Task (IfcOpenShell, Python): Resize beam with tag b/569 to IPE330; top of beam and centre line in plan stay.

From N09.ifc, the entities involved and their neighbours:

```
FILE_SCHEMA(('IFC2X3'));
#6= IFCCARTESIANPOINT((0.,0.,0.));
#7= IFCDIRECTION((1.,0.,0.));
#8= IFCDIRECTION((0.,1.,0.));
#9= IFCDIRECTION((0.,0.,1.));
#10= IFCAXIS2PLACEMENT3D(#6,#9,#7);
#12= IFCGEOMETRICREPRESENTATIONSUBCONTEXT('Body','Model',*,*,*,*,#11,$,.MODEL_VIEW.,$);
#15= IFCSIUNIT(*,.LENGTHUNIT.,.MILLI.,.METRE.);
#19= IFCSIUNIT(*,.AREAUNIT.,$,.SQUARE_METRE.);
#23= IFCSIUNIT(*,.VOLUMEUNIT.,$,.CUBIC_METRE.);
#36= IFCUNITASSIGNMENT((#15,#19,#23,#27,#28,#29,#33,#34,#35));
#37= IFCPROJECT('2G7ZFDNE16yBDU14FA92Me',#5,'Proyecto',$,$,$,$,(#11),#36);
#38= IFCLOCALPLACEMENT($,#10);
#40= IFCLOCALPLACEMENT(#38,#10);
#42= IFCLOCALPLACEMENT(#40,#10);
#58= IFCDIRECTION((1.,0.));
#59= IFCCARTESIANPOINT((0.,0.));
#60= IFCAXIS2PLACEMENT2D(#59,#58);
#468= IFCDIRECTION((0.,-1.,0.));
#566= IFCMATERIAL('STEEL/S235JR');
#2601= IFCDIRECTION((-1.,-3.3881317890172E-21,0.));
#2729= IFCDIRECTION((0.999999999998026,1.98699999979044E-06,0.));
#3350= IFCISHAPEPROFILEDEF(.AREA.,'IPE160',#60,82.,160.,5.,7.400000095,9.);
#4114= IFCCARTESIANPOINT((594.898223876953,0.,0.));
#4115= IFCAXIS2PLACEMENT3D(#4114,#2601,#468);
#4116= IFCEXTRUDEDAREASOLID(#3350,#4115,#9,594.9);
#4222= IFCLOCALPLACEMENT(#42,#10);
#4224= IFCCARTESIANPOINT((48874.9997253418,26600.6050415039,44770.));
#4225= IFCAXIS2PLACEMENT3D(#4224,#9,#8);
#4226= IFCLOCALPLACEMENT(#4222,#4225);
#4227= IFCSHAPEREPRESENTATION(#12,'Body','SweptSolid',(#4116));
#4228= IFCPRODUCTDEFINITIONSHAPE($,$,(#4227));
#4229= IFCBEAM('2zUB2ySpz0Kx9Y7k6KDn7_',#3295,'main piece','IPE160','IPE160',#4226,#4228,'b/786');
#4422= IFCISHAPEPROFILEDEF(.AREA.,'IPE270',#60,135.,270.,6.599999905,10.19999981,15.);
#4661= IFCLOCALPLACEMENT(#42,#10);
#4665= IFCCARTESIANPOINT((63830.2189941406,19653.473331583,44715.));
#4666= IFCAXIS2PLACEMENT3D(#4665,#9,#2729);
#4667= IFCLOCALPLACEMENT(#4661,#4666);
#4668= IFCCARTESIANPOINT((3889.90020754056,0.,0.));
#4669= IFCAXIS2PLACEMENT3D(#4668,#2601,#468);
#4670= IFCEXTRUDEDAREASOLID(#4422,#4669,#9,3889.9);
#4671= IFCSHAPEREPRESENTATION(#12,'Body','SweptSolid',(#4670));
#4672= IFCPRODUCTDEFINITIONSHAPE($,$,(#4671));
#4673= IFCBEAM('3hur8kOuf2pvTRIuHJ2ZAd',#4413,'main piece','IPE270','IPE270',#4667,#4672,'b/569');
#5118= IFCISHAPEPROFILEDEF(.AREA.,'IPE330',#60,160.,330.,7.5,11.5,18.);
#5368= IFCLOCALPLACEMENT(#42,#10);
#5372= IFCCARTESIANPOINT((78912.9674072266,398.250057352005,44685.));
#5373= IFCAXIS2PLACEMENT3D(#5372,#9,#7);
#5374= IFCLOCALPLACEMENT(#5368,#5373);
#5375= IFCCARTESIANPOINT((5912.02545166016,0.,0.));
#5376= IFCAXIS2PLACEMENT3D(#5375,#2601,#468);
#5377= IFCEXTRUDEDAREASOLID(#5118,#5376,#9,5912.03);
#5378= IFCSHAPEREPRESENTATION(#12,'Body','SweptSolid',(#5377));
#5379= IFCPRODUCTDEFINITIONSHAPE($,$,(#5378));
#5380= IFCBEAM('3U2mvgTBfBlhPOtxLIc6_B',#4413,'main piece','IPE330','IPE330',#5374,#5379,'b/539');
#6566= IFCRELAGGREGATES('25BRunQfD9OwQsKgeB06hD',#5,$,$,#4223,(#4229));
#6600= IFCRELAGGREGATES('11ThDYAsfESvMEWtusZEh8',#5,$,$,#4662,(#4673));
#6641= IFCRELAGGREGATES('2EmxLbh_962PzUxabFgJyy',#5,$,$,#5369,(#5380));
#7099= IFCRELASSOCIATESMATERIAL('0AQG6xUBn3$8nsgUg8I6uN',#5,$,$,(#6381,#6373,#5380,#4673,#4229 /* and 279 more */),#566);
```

```python
import ifcopenshell
import ifcopenshell.util.element
import ifcopenshell.util.representation

model = ifcopenshell.open("N09.ifc")

member = model.by_guid("3hur8kOuf2pvTRIuHJ2ZAd")
source = next(p for p in model.by_type("IfcIShapeProfileDef") if p.ProfileName == "IPE330")

body = ifcopenshell.util.representation.get_representation(member, "Model", "Body")
solid = body.Items[0]
old_profile = solid.SweptArea

# Copy the section's sizes but keep this member's own profile position.
profile = ifcopenshell.util.element.copy(model, source)
# Profiles are centred, so shift by half the change in depth to hold the top.
shift = (old_profile.OverallDepth - profile.OverallDepth) / 2
x, y = old_profile.Position.Location.Coordinates
up = (0.0, 1.0)  # upwards, in the solid's own plane
location = model.createIfcCartesianPoint((x + up[0] * shift, y + up[1] * shift))
profile.Position = model.createIfcAxis2Placement2D(location, old_profile.Position.RefDirection)
solid.SweptArea = profile
if not model.get_total_inverses(old_profile):
    ifcopenshell.util.element.remove_deep2(model, old_profile)
member.Description = member.Description.replace("IPE270", "IPE330")
member.ObjectType = member.ObjectType.replace("IPE270", "IPE330")

print(solid.SweptArea)

model.write("N09_rev.ifc")
```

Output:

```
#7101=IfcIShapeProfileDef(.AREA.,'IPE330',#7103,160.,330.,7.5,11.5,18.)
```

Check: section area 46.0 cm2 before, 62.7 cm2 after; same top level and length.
